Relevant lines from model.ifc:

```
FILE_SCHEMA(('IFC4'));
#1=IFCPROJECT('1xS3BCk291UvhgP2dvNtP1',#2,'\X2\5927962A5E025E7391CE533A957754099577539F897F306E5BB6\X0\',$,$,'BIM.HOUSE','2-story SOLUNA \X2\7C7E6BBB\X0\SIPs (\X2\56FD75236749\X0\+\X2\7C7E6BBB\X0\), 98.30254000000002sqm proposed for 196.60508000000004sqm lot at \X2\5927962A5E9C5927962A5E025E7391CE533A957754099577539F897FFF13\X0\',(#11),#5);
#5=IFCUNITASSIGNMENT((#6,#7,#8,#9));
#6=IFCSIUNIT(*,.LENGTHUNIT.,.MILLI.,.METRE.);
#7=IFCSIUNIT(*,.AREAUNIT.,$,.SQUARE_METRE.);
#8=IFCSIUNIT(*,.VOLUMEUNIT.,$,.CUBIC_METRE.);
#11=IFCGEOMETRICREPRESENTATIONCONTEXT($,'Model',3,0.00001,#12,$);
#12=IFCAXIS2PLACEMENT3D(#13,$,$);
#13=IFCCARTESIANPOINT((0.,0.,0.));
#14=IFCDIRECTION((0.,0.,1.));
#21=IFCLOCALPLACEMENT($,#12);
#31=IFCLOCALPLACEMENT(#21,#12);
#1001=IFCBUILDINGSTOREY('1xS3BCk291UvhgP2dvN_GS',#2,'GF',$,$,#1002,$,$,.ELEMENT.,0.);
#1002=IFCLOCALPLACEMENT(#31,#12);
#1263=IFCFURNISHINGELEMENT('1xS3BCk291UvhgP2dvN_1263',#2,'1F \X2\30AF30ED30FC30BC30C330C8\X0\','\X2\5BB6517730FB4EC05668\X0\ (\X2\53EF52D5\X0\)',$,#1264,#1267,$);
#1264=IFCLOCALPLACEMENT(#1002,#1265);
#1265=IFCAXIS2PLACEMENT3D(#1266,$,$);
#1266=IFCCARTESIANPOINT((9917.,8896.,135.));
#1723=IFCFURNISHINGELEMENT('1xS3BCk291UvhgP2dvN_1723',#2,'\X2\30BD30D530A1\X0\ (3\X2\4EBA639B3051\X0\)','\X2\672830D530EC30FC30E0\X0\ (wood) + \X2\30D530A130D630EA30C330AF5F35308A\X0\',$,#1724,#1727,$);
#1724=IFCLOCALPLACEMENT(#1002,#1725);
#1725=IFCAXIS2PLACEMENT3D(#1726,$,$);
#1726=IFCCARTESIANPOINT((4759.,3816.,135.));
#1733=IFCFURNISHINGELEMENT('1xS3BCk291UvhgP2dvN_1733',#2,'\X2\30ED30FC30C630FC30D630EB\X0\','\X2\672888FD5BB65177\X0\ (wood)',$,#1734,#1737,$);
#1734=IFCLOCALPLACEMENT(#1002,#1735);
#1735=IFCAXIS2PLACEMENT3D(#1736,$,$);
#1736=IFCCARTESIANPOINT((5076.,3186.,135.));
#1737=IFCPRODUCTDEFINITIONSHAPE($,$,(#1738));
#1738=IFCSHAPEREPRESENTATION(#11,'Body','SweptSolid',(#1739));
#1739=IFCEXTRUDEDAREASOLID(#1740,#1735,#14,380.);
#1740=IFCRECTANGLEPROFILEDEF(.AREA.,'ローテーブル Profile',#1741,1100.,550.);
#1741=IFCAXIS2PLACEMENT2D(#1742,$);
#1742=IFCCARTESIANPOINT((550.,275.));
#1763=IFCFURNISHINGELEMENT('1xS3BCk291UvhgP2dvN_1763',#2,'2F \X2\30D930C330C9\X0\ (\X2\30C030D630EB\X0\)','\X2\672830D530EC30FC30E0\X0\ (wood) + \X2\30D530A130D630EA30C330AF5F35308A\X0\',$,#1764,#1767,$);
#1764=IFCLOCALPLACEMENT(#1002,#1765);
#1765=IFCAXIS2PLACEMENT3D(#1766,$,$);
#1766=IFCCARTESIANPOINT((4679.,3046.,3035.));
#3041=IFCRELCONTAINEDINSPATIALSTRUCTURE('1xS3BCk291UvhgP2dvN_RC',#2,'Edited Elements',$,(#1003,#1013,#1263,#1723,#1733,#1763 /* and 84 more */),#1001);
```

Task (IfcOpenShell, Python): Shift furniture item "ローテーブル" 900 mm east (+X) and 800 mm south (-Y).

```python
import ifcopenshell
import ifcopenshell.api.geometry
import ifcopenshell.util.placement
import ifcopenshell.util.unit

model = ifcopenshell.open("model.ifc")
unit_scale = ifcopenshell.util.unit.calculate_unit_scale(model)

item = model.by_guid("1xS3BCk291UvhgP2dvN_1733")
matrix = ifcopenshell.util.placement.get_local_placement(item.ObjectPlacement)
matrix[0, 3] += 0.9 / unit_scale
matrix[1, 3] -= 0.8 / unit_scale
ifcopenshell.api.geometry.edit_object_placement(model, product=item, matrix=matrix, is_si=False)

print(ifcopenshell.util.placement.get_local_placement(item.ObjectPlacement).round(3) + 0.0)

model.write("model_updated.ifc")
```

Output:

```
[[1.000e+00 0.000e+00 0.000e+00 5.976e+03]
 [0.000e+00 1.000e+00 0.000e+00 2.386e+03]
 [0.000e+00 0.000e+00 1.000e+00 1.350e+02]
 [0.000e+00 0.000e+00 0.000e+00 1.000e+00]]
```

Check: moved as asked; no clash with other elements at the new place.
